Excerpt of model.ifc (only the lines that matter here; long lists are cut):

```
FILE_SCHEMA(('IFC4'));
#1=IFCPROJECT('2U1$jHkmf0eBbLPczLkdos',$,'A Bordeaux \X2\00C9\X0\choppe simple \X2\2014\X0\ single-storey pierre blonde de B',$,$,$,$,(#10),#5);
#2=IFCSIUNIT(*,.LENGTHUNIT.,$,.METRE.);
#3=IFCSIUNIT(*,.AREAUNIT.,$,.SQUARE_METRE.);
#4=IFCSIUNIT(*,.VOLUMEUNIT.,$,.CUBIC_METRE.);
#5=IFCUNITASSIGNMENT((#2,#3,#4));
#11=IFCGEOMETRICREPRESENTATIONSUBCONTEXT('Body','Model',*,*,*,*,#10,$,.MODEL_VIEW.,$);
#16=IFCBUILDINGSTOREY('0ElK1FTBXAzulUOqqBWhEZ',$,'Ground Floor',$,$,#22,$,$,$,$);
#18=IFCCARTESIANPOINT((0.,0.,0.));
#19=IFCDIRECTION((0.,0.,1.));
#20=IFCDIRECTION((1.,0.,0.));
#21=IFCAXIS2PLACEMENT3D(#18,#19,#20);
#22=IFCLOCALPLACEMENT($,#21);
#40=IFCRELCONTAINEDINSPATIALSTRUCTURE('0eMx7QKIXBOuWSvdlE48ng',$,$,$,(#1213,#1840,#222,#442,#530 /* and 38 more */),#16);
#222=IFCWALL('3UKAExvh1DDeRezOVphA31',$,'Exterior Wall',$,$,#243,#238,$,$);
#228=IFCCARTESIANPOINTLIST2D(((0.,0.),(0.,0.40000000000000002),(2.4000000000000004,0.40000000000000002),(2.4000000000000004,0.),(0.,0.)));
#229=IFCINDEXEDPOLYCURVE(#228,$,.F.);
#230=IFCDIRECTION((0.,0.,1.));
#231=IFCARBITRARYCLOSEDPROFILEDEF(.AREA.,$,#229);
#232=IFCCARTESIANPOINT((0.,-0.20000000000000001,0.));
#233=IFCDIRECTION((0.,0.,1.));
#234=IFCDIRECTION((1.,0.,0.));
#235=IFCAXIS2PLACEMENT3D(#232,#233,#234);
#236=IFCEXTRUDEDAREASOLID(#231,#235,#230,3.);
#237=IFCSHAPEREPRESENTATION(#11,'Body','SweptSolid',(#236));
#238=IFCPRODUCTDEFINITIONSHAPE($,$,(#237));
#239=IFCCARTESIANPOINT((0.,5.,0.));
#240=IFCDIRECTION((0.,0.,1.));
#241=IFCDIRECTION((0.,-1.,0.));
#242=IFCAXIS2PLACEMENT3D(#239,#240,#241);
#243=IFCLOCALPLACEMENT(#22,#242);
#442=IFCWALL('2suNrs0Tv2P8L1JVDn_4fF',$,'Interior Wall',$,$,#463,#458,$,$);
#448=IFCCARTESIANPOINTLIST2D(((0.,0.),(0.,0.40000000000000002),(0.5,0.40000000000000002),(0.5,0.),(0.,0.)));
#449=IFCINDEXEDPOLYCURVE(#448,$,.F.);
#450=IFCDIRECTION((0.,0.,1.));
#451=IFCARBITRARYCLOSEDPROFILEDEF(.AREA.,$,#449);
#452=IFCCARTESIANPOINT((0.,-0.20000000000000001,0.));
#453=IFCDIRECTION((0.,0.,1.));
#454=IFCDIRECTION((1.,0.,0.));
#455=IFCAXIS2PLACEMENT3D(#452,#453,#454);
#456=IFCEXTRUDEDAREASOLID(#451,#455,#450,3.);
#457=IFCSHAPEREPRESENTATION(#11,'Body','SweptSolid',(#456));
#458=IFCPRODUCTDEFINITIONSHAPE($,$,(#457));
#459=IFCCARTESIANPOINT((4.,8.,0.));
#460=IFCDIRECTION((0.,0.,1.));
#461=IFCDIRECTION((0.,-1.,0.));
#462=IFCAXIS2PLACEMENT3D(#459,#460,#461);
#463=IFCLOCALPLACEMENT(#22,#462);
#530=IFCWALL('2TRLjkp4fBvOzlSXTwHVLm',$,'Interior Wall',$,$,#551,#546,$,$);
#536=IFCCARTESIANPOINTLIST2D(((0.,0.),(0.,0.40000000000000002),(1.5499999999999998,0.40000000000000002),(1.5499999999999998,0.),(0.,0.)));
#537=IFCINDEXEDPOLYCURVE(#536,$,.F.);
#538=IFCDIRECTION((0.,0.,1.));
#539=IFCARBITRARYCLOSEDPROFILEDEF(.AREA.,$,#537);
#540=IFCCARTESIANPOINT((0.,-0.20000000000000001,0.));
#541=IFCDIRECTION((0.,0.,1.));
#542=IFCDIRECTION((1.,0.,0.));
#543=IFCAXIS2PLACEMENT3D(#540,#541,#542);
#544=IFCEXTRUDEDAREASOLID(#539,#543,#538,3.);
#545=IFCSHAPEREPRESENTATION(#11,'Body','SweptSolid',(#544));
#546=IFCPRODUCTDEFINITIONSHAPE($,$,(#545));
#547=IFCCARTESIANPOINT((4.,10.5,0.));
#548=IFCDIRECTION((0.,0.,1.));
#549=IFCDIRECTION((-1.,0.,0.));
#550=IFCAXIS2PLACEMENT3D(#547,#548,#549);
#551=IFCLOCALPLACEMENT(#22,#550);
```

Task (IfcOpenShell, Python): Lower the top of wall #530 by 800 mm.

```python
import ifcopenshell
import ifcopenshell.geom
import ifcopenshell.util.representation
import ifcopenshell.util.shape
import ifcopenshell.util.unit

model = ifcopenshell.open("model.ifc")
unit_scale = ifcopenshell.util.unit.calculate_unit_scale(model)
settings = ifcopenshell.geom.settings()


def volume(element):
    """Net volume in cubic metres, openings subtracted."""
    shape = ifcopenshell.geom.create_shape(settings, element)
    return ifcopenshell.util.shape.get_volume(shape.geometry)


wall = model.by_guid("2TRLjkp4fBvOzlSXTwHVLm")
before = volume(wall)

body = ifcopenshell.util.representation.get_representation(wall, "Model", "Body")
solid = body.Items[0]
old_height = solid.Depth
solid.Depth -= 0.8 / unit_scale
after = volume(wall)

print(f"height {old_height:g} -> {solid.Depth:g}, volume {before:.3f} -> {after:.3f} m3")

model.write("model-out.ifc")
```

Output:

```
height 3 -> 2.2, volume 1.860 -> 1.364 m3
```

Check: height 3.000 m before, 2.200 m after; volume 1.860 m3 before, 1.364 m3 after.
